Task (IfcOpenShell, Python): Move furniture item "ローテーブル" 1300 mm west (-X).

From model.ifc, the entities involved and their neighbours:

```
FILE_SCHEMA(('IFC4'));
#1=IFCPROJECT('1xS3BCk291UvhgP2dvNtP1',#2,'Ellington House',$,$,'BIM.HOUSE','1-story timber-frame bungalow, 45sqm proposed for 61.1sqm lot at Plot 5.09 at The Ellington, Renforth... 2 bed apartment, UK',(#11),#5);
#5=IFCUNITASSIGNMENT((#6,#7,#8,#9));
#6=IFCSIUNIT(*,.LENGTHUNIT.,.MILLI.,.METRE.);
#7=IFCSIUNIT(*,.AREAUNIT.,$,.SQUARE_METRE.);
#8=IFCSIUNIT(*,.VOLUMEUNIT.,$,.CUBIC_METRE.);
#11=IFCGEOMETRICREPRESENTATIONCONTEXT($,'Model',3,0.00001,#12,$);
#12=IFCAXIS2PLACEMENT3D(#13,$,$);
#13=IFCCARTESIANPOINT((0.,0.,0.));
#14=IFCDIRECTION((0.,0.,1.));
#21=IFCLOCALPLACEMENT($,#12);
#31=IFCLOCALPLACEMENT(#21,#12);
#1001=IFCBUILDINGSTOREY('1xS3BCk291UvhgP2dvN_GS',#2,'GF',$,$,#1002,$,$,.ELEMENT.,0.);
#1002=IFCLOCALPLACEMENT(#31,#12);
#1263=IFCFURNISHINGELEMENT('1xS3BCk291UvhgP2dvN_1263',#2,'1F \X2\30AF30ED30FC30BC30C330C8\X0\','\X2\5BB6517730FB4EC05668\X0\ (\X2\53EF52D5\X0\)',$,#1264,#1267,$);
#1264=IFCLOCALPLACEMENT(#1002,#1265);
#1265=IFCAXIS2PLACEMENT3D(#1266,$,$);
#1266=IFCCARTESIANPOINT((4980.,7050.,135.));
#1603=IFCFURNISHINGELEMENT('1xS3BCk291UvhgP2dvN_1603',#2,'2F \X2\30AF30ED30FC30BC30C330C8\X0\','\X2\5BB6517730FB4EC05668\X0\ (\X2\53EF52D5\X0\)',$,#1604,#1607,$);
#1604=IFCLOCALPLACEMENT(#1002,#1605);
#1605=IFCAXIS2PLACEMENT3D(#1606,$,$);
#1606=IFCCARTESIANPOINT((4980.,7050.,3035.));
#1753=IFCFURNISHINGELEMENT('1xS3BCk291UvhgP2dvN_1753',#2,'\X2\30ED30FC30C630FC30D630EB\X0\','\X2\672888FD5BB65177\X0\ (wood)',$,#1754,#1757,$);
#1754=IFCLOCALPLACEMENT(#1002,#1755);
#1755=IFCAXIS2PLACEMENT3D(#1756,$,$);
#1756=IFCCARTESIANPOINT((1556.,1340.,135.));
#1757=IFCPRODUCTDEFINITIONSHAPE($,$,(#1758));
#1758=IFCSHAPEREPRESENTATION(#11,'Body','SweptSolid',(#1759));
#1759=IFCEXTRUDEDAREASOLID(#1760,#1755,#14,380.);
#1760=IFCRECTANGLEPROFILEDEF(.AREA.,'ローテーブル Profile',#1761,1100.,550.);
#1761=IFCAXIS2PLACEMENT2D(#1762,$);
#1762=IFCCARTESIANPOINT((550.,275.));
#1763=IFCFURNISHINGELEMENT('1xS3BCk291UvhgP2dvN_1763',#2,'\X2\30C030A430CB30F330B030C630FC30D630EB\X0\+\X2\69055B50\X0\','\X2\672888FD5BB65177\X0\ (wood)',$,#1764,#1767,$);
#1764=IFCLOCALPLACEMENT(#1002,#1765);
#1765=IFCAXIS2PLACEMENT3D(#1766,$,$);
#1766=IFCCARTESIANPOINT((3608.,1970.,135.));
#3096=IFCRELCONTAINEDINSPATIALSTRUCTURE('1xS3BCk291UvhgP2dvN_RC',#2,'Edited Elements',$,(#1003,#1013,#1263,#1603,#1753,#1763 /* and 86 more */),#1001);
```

```python
import ifcopenshell
import ifcopenshell.api.geometry
import ifcopenshell.util.placement
import ifcopenshell.util.unit

model = ifcopenshell.open("model.ifc")
unit_scale = ifcopenshell.util.unit.calculate_unit_scale(model)

item = model.by_id(1753)
matrix = ifcopenshell.util.placement.get_local_placement(item.ObjectPlacement)
matrix[0, 3] -= 1.3 / unit_scale
ifcopenshell.api.geometry.edit_object_placement(model, product=item, matrix=matrix, is_si=False)

print(ifcopenshell.util.placement.get_local_placement(item.ObjectPlacement).round(3) + 0.0)

model.write("model_rev.ifc")
```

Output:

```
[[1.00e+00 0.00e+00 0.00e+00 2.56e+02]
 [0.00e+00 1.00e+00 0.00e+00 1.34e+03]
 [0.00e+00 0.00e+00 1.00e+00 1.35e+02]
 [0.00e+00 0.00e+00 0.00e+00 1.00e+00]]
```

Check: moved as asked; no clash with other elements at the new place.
